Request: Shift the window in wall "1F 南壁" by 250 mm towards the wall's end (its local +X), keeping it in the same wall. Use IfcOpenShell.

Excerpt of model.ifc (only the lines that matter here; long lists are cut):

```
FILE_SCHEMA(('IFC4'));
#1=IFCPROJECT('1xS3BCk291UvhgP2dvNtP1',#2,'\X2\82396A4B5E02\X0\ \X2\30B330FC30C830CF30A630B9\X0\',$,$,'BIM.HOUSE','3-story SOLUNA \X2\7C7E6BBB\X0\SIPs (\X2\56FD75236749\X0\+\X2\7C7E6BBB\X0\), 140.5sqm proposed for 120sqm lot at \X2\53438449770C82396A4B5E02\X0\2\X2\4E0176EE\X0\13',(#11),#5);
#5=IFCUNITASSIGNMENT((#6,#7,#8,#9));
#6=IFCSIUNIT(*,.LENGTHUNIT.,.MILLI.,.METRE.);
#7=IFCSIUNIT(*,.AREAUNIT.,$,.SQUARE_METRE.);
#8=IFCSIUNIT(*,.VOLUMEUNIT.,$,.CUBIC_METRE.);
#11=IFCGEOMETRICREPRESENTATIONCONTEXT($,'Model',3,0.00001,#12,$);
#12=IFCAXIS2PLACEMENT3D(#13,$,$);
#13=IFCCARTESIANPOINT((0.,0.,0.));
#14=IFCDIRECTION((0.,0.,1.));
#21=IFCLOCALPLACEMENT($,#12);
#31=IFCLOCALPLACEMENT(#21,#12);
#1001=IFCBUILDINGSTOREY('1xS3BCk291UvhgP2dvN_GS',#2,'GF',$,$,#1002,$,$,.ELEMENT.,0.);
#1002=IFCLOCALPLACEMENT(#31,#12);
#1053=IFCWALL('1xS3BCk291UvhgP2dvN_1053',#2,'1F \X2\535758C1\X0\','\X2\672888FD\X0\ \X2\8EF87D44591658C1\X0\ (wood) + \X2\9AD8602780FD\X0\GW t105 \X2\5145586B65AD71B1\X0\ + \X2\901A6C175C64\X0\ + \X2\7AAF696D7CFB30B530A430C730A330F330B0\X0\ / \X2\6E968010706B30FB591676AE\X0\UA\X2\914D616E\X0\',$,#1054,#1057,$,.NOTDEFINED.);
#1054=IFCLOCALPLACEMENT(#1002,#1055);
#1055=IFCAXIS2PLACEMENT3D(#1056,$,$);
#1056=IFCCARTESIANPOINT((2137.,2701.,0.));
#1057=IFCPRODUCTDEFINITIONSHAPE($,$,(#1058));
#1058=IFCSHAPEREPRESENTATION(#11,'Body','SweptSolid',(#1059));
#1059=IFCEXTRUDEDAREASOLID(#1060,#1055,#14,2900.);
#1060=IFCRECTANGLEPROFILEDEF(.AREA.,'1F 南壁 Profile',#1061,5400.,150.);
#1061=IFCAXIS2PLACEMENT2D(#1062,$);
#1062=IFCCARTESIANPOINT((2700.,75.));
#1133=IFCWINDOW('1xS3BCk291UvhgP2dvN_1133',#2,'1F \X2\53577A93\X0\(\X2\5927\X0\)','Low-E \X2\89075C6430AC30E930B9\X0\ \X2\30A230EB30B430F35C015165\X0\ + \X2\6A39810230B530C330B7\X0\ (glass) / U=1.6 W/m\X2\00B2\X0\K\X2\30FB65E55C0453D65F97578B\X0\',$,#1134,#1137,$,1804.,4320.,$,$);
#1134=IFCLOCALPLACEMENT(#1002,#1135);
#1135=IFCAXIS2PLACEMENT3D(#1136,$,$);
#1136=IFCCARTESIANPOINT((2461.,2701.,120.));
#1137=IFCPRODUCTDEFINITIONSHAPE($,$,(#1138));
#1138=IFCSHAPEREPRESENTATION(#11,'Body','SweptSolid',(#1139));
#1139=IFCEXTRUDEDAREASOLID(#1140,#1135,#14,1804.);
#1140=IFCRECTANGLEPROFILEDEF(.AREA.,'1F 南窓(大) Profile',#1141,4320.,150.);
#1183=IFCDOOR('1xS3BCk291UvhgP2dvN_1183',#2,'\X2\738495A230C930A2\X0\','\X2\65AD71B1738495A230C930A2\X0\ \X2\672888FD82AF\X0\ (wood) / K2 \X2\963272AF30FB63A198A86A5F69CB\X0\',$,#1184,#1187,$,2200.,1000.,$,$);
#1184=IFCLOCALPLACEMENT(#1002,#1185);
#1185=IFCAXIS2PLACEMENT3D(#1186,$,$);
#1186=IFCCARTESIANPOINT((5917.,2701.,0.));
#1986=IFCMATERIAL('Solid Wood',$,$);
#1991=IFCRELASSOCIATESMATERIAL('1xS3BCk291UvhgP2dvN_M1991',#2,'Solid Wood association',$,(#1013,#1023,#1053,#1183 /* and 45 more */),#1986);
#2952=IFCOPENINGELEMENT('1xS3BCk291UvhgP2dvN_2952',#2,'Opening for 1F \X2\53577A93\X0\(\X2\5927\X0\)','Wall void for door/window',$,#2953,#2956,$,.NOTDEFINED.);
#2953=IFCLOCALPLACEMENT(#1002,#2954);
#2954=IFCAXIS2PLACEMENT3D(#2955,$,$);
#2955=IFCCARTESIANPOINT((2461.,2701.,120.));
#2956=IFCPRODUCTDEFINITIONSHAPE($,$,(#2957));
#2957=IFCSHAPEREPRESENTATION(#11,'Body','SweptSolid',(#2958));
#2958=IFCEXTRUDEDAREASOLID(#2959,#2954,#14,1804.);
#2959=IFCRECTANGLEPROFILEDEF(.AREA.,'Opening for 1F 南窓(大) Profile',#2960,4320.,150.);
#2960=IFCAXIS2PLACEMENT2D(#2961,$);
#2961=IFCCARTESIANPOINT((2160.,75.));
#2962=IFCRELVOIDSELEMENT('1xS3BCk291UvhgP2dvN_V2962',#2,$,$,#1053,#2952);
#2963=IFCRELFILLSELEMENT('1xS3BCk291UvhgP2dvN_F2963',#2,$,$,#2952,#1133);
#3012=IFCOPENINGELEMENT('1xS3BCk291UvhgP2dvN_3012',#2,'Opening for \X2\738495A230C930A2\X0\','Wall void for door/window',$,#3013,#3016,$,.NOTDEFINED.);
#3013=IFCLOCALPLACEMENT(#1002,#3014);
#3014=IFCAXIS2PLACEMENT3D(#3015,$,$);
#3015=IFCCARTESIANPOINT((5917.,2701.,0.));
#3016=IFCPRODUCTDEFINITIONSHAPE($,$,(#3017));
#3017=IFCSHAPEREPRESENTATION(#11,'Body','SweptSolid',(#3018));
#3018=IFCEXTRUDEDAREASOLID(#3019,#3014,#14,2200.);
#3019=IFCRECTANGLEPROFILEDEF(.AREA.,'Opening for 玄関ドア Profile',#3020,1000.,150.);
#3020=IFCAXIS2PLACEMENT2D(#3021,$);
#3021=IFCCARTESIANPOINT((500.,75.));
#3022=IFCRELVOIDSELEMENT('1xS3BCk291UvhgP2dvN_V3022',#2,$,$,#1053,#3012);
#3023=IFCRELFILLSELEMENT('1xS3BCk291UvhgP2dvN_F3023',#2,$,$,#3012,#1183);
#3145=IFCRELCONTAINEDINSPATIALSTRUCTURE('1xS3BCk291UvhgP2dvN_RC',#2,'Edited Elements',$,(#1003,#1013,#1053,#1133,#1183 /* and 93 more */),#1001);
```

```python
import ifcopenshell
import ifcopenshell.api.geometry
import ifcopenshell.util.placement
import ifcopenshell.util.unit

model = ifcopenshell.open("model.ifc")
unit_scale = ifcopenshell.util.unit.calculate_unit_scale(model)

window = model.by_id(1133)
opening = window.FillsVoids[0].RelatingOpeningElement
wall = opening.VoidsElements[0].RelatingBuildingElement

wall_matrix = ifcopenshell.util.placement.get_local_placement(wall.ObjectPlacement)
shift = wall_matrix[:3, 0] * 0.25 / unit_scale
before = ifcopenshell.util.placement.get_local_placement(window.ObjectPlacement)[:3, 3].copy()

# The window is not placed relative to its opening, so move both.
for product in (opening, window):
    matrix = ifcopenshell.util.placement.get_local_placement(product.ObjectPlacement)
    matrix[:3, 3] += shift
    ifcopenshell.api.geometry.edit_object_placement(model, product=product, matrix=matrix, is_si=False)

after = ifcopenshell.util.placement.get_local_placement(window.ObjectPlacement)[:3, 3]
print("window moved by", (after - before).round(3) + 0.0)

model.write("model_updated.ifc")
```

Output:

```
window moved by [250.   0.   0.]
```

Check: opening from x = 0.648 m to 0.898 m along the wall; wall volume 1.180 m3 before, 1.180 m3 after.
